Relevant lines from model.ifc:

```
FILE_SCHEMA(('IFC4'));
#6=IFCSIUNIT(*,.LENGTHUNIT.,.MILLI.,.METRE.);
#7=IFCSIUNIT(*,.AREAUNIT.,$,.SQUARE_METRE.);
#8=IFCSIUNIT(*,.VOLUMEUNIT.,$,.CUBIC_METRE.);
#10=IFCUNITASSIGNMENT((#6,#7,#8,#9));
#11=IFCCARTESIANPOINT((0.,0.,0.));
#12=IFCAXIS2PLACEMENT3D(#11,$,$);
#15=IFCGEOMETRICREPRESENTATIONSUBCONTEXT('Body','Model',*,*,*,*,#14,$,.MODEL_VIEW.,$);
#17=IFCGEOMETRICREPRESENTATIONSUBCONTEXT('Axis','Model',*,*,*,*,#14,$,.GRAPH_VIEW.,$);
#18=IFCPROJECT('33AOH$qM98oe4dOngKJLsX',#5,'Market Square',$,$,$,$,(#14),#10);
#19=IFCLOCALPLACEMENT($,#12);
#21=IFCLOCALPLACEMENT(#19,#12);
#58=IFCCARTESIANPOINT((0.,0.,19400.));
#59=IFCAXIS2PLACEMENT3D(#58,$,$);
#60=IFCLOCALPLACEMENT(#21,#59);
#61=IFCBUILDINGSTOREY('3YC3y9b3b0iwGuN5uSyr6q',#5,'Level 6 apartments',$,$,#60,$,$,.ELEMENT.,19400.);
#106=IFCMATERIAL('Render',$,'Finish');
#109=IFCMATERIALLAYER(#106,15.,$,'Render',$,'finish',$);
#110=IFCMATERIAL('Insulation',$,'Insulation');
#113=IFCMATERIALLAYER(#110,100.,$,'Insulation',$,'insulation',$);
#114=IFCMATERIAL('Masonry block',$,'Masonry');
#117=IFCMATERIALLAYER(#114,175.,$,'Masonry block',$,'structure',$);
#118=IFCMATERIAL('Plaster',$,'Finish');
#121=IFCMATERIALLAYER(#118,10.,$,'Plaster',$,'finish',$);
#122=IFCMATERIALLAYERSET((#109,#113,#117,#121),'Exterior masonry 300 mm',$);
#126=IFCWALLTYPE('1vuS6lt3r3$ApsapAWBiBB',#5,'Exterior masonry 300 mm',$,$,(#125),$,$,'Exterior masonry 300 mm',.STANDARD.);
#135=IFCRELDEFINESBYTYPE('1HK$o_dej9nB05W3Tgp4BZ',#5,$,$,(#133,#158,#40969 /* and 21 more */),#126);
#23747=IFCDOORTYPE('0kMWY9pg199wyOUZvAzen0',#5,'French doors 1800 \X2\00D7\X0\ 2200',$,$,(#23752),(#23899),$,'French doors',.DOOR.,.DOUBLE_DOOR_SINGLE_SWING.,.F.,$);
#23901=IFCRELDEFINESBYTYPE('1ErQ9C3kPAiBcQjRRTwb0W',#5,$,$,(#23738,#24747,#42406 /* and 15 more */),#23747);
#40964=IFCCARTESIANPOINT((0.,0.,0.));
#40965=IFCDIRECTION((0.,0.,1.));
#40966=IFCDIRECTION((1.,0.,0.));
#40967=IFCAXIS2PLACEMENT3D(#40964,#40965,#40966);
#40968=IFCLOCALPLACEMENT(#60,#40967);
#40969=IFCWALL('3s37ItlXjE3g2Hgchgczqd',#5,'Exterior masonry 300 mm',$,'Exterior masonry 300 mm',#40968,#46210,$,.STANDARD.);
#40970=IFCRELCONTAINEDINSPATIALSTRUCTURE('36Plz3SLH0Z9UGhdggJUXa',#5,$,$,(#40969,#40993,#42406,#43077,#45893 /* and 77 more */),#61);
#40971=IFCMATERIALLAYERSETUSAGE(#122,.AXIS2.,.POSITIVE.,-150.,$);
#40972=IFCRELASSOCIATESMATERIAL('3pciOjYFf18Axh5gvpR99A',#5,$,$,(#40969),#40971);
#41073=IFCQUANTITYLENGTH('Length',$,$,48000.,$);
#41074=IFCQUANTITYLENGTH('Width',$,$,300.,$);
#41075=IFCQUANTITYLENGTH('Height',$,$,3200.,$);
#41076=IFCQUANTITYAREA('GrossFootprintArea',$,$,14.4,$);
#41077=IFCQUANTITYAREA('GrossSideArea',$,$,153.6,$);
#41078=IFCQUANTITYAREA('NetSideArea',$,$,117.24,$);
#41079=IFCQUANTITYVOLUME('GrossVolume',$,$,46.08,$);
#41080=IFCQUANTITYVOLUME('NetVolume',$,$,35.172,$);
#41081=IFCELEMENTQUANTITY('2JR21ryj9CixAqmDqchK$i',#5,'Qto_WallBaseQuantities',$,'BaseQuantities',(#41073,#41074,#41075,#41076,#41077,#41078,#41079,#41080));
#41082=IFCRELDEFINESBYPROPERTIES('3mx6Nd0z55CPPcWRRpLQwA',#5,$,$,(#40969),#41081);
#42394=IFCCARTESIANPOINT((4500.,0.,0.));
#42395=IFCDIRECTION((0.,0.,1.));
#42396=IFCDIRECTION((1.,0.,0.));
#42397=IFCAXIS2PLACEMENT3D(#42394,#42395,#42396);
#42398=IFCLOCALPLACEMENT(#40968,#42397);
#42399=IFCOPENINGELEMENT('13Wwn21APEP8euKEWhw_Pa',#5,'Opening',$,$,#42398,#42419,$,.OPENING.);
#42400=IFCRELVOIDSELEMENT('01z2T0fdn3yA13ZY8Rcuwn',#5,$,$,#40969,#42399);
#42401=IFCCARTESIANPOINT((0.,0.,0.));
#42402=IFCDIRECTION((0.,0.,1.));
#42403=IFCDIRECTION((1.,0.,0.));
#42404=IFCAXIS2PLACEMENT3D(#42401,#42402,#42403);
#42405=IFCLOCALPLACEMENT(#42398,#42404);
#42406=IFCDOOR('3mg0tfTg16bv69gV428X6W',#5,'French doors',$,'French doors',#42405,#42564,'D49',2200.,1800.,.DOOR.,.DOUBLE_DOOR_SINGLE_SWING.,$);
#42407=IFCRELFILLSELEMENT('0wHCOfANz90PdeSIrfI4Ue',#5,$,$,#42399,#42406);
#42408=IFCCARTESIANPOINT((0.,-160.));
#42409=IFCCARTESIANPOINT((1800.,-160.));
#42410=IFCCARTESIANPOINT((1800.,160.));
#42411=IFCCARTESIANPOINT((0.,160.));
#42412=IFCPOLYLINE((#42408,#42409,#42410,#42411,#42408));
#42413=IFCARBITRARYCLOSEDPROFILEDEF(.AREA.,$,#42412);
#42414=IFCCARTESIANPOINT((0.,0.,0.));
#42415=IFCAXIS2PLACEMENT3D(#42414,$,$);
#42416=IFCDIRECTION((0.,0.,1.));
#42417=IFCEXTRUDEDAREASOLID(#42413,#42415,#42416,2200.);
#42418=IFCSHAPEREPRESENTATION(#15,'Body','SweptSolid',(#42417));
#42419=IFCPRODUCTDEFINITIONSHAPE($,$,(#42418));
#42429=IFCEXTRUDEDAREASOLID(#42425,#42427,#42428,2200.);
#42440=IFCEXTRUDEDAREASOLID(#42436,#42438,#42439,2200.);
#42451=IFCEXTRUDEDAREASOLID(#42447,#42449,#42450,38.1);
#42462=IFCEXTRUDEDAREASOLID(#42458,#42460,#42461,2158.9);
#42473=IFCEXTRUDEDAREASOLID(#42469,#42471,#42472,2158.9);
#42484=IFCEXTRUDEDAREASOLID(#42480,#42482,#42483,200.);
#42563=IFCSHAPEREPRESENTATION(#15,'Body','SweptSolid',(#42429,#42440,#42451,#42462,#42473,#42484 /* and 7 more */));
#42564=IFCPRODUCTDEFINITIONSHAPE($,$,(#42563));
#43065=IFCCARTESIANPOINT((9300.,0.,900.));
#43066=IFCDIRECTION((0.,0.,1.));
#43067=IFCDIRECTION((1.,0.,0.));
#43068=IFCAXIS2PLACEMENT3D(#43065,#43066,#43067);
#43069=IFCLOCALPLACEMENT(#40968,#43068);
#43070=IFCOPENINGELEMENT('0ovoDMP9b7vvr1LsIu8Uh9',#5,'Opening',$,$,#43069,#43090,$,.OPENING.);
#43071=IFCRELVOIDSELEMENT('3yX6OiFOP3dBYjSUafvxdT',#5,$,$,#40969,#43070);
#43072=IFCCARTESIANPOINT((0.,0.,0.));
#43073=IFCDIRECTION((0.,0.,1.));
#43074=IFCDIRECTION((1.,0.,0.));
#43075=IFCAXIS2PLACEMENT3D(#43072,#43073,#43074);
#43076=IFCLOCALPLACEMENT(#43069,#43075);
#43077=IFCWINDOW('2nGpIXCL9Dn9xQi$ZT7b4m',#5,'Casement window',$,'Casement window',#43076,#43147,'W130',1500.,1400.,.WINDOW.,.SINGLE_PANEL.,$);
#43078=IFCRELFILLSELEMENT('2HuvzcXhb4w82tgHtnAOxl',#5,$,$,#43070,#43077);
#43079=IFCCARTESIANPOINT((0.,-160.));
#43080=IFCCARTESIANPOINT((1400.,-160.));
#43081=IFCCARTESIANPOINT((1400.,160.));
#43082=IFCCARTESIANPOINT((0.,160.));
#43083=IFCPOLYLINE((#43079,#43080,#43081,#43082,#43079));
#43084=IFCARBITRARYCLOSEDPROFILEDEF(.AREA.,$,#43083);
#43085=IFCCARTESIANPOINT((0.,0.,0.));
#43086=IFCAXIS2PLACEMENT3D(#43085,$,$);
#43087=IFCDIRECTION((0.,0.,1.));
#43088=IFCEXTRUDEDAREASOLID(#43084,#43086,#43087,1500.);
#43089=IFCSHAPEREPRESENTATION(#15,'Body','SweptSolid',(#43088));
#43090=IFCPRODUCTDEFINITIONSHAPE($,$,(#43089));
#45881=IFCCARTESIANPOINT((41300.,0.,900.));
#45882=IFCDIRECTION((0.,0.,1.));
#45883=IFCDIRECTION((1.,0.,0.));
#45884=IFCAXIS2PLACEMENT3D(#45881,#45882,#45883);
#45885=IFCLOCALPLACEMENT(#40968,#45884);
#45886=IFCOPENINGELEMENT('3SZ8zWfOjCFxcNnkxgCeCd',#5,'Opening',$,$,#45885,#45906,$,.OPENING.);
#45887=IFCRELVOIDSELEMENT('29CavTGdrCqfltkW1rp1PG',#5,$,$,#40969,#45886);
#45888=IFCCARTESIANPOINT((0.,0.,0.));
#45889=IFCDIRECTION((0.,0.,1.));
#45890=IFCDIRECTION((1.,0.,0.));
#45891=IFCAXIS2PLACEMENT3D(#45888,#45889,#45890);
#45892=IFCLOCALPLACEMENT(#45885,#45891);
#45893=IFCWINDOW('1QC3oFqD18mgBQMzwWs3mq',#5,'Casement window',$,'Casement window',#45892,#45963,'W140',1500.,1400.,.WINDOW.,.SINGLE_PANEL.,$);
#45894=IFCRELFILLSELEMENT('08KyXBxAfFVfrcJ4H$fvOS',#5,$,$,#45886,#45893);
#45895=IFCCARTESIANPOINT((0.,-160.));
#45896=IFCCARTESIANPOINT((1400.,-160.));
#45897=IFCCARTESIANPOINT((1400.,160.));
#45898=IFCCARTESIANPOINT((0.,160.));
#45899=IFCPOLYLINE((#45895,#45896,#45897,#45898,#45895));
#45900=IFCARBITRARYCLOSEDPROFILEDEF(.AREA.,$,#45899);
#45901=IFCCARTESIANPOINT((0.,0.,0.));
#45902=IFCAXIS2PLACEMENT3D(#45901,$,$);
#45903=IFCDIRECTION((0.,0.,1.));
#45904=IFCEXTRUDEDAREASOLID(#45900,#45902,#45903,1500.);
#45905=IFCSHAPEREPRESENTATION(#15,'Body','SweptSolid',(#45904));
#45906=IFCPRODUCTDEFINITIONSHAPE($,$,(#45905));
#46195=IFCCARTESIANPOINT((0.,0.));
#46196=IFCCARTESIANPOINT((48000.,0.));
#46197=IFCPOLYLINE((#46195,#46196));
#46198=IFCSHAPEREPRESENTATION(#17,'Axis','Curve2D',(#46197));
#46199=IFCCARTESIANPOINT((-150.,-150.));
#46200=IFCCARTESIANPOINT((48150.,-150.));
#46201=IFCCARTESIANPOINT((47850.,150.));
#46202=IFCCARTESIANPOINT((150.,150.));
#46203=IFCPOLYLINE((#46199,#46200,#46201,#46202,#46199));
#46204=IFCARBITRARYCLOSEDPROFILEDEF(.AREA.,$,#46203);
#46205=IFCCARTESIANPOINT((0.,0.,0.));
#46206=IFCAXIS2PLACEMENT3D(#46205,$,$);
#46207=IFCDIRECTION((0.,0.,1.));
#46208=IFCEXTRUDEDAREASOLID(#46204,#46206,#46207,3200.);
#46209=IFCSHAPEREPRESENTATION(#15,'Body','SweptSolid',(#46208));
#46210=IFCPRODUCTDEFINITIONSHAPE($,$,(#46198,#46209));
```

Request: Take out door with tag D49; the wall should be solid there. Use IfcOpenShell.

```python
import ifcopenshell
import ifcopenshell.api.feature
import ifcopenshell.api.pset
import ifcopenshell.api.root
import ifcopenshell.geom
import ifcopenshell.util.element
import ifcopenshell.util.shape
import ifcopenshell.util.unit

model = ifcopenshell.open("model.ifc")
area_scale = ifcopenshell.util.unit.calculate_unit_scale(model, "AREAUNIT")
volume_scale = ifcopenshell.util.unit.calculate_unit_scale(model, "VOLUMEUNIT")
settings = ifcopenshell.geom.settings()


def volume(element):
    """Net volume in cubic metres, openings subtracted."""
    shape = ifcopenshell.geom.create_shape(settings, element)
    return ifcopenshell.util.shape.get_volume(shape.geometry)


door = model.by_guid("3mg0tfTg16bv69gV428X6W")
opening = door.FillsVoids[0].RelatingOpeningElement
wall = opening.VoidsElements[0].RelatingBuildingElement
before = volume(wall)

ifcopenshell.api.root.remove_product(model, product=door)
ifcopenshell.api.feature.remove_feature(model, feature=opening)

after = volume(wall)
thickness = 0.3  # wall thickness in metres

# Update the wall's stored quantities.
qto = model.by_id(ifcopenshell.util.element.get_pset(wall, "Qto_WallBaseQuantities", should_inherit=False)["id"])
ifcopenshell.api.pset.edit_qto(model, qto=qto, properties={
    "NetSideArea": after / thickness / area_scale,
    "NetVolume": after / volume_scale,
})

print(f"wall volume {before:.3f} -> {after:.3f} m3")

model.write("model_rev.ifc")
```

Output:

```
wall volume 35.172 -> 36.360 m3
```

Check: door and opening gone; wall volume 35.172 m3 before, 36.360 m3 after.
